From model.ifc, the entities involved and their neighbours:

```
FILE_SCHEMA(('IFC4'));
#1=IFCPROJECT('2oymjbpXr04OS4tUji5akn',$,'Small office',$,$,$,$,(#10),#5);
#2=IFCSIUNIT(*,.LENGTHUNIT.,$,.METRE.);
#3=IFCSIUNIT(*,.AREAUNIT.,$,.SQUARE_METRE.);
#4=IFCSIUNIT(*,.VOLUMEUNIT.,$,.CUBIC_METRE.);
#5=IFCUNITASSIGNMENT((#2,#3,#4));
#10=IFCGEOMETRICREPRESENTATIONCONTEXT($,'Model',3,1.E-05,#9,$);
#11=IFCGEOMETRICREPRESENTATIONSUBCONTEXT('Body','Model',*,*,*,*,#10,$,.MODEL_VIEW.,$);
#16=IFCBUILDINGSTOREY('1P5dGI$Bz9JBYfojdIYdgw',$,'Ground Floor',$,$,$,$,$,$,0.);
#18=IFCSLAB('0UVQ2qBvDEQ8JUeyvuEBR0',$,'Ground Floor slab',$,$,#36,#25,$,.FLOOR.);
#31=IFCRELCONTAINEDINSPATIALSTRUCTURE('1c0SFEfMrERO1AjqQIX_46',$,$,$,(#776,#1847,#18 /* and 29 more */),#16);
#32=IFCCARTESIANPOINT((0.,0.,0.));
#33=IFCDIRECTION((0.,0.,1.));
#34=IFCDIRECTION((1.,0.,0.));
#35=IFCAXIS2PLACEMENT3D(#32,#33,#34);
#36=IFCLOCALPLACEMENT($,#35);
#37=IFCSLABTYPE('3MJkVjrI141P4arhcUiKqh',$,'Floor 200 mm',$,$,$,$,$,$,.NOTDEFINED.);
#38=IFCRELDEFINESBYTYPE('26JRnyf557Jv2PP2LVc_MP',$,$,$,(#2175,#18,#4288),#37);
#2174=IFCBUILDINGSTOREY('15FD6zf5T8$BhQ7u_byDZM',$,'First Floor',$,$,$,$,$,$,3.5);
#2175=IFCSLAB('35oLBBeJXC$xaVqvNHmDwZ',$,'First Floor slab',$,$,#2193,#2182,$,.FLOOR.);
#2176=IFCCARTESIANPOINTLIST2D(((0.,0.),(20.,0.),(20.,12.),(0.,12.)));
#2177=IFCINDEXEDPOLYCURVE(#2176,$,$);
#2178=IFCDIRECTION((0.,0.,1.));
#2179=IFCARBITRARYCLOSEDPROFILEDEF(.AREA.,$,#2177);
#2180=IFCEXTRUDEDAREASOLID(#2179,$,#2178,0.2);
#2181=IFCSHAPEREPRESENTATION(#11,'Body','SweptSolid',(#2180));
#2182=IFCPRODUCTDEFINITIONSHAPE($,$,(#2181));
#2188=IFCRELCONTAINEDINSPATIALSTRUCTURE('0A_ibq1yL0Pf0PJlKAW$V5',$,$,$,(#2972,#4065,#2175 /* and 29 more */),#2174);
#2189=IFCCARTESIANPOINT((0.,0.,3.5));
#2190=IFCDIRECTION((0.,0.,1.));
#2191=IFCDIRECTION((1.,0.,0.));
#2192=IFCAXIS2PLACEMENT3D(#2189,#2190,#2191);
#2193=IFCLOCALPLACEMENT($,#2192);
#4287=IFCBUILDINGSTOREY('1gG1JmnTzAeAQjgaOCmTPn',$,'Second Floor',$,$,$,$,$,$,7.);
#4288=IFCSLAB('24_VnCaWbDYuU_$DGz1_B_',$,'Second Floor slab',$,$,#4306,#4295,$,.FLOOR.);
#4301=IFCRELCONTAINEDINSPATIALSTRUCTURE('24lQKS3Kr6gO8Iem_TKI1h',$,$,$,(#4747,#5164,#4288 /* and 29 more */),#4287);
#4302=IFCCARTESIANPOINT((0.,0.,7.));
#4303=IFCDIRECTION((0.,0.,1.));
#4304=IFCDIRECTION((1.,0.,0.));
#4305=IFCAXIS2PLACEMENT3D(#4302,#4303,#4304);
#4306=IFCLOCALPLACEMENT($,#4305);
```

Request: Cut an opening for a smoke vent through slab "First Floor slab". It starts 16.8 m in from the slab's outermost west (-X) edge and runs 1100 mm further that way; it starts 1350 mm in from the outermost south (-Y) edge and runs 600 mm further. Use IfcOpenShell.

```python
import numpy as np
import ifcopenshell
import ifcopenshell.api.feature
import ifcopenshell.api.geometry
import ifcopenshell.api.root
import ifcopenshell.geom
import ifcopenshell.util.placement
import ifcopenshell.util.representation
import ifcopenshell.util.shape
import ifcopenshell.util.unit

model = ifcopenshell.open("model.ifc")
unit_scale = ifcopenshell.util.unit.calculate_unit_scale(model)
settings = ifcopenshell.geom.settings()


def volume(element):
    """Net volume in cubic metres, openings subtracted."""
    shape = ifcopenshell.geom.create_shape(settings, element)
    return ifcopenshell.util.shape.get_volume(shape.geometry)


slab = model.by_guid("35oLBBeJXC$xaVqvNHmDwZ")
before = volume(slab)

# Extent in the slab's own axes, in metres. The edges named are its -X and -Y sides.
slab_shape = ifcopenshell.geom.create_shape(settings, slab)
vertices = ifcopenshell.util.shape.get_vertices(slab_shape.geometry)
x_min, y_min, bottom = vertices.min(axis=0)
top = vertices[:, 2].max()

opening = ifcopenshell.api.root.create_entity(model, ifc_class="IfcOpeningElement", name="Smoke vent opening", predefined_type="OPENING")
context = ifcopenshell.util.representation.get_context(model, "Model", "Body", "MODEL_VIEW")
width, depth = 1.1, 0.6
outline = [(0.0, 0.0), (width, 0.0), (width, depth), (0.0, depth), (0.0, 0.0)]
# Overshoot both faces by 50 mm so the cut is clean.
shape = ifcopenshell.api.geometry.add_slab_representation(
    model, context=context, depth=top - bottom + 0.1, polyline=outline
)
ifcopenshell.api.geometry.assign_representation(model, product=opening, representation=shape)

matrix = ifcopenshell.util.placement.get_local_placement(slab.ObjectPlacement)
matrix[:, 3] = matrix @ np.append(np.array([x_min + 16.8, y_min + 1.35, bottom - 0.05]) / unit_scale, 1.0)
ifcopenshell.api.geometry.edit_object_placement(model, product=opening, matrix=matrix, is_si=False)
ifcopenshell.api.feature.add_feature(model, feature=opening, element=slab)

after = volume(slab)

print(f"slab volume {before:.3f} -> {after:.3f} m3")

model.write("model-out.ifc")
```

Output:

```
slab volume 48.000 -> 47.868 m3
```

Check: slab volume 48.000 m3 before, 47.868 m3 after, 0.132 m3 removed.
